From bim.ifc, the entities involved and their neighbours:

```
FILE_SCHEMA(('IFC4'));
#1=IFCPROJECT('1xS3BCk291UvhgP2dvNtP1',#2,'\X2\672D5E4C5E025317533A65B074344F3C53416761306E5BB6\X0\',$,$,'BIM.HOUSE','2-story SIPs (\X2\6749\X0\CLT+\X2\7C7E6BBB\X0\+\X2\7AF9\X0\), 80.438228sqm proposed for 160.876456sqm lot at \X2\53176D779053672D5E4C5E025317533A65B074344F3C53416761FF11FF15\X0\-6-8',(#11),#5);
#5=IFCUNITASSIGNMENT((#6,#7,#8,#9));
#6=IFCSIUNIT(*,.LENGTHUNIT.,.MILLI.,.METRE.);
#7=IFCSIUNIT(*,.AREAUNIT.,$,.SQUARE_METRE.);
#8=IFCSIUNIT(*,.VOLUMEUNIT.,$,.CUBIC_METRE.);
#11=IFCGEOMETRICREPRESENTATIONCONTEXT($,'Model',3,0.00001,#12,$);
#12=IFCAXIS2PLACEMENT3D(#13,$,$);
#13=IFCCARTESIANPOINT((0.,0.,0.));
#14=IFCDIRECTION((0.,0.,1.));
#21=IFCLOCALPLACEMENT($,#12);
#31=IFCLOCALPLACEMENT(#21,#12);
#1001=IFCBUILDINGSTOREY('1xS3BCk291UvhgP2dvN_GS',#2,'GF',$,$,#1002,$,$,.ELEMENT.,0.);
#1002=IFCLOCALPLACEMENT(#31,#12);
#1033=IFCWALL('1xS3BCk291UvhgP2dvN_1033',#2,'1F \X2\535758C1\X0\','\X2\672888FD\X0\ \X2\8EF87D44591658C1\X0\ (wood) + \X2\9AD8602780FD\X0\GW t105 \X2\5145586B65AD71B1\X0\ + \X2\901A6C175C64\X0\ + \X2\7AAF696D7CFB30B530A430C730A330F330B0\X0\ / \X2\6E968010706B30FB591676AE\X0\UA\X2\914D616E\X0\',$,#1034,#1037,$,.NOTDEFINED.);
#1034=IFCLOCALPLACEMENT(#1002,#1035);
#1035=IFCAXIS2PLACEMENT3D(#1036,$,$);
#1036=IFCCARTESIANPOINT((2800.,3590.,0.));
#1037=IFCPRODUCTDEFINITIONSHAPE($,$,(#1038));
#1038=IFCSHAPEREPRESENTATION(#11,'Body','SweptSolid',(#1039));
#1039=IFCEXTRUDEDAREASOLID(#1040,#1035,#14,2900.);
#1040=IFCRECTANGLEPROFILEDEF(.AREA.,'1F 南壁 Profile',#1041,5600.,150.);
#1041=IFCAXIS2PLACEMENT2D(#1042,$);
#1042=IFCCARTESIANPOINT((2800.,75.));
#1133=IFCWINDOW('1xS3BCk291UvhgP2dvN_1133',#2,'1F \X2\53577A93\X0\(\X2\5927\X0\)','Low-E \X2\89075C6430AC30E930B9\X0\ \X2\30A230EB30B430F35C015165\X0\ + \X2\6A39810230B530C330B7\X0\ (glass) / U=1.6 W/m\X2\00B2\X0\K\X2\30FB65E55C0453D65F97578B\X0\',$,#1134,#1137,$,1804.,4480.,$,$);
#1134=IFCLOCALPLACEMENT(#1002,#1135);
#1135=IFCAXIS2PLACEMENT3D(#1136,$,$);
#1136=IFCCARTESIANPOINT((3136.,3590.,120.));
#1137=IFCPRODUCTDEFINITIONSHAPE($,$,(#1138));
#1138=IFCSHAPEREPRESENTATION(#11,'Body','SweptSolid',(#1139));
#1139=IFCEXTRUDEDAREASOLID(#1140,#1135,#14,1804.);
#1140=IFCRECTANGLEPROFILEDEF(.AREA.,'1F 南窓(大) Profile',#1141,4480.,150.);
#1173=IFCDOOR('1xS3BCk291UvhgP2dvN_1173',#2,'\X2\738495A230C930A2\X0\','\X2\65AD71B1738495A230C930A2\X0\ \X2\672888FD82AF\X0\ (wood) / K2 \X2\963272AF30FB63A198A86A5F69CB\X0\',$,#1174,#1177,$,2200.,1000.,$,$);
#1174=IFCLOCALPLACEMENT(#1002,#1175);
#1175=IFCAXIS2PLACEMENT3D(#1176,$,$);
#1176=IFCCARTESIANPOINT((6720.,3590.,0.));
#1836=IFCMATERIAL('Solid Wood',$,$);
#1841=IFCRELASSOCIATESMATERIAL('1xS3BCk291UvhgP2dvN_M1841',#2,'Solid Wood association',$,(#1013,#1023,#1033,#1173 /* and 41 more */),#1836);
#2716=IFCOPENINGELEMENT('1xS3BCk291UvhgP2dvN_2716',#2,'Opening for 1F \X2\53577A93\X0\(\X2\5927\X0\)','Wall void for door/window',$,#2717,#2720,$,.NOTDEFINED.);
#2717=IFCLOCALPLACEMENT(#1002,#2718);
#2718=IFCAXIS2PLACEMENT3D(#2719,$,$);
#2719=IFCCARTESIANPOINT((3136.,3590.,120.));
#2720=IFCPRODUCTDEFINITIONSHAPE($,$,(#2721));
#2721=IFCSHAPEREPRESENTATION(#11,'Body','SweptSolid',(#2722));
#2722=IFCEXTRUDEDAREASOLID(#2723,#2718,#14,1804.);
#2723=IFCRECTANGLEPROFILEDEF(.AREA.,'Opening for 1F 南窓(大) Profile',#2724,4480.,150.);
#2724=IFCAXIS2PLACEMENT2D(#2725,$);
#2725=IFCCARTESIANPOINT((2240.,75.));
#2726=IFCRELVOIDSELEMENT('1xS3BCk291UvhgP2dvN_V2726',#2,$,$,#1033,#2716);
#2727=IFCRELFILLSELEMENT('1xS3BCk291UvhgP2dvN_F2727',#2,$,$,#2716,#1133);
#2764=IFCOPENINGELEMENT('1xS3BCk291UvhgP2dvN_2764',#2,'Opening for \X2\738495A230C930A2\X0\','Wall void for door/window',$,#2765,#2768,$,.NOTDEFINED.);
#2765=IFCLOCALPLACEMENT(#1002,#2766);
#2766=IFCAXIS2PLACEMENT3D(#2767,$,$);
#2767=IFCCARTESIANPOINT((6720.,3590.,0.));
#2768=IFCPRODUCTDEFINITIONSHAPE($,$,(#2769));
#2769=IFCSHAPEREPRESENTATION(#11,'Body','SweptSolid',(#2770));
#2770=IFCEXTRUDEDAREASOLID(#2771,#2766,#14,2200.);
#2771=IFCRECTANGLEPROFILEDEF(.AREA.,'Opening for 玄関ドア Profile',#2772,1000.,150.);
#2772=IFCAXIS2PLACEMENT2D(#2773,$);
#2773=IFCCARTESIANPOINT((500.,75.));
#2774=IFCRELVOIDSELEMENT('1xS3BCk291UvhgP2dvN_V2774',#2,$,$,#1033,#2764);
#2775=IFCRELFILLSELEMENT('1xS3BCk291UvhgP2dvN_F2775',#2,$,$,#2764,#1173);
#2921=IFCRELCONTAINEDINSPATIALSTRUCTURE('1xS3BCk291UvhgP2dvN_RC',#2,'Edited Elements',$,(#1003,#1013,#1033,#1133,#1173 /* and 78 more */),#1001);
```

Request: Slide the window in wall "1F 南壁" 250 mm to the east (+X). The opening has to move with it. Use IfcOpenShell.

```python
import ifcopenshell
import ifcopenshell.api.geometry
import ifcopenshell.util.placement

model = ifcopenshell.open("bim.ifc")

window = model.by_guid("1xS3BCk291UvhgP2dvN_1133")
opening = window.FillsVoids[0].RelatingOpeningElement
wall = opening.VoidsElements[0].RelatingBuildingElement

wall_matrix = ifcopenshell.util.placement.get_local_placement(wall.ObjectPlacement)
shift = wall_matrix[:3, 0] * 250.0
before = ifcopenshell.util.placement.get_local_placement(window.ObjectPlacement)[:3, 3].copy()

# The window is not placed relative to its opening, so move both.
for product in (opening, window):
    matrix = ifcopenshell.util.placement.get_local_placement(product.ObjectPlacement)
    matrix[:3, 3] += shift
    ifcopenshell.api.geometry.edit_object_placement(model, product=product, matrix=matrix, is_si=False)

after = ifcopenshell.util.placement.get_local_placement(window.ObjectPlacement)[:3, 3]
print("window moved by", (after - before).round(3) + 0.0)

model.write("bim_rev.ifc")
```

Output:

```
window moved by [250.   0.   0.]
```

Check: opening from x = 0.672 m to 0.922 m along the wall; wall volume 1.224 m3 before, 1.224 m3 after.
